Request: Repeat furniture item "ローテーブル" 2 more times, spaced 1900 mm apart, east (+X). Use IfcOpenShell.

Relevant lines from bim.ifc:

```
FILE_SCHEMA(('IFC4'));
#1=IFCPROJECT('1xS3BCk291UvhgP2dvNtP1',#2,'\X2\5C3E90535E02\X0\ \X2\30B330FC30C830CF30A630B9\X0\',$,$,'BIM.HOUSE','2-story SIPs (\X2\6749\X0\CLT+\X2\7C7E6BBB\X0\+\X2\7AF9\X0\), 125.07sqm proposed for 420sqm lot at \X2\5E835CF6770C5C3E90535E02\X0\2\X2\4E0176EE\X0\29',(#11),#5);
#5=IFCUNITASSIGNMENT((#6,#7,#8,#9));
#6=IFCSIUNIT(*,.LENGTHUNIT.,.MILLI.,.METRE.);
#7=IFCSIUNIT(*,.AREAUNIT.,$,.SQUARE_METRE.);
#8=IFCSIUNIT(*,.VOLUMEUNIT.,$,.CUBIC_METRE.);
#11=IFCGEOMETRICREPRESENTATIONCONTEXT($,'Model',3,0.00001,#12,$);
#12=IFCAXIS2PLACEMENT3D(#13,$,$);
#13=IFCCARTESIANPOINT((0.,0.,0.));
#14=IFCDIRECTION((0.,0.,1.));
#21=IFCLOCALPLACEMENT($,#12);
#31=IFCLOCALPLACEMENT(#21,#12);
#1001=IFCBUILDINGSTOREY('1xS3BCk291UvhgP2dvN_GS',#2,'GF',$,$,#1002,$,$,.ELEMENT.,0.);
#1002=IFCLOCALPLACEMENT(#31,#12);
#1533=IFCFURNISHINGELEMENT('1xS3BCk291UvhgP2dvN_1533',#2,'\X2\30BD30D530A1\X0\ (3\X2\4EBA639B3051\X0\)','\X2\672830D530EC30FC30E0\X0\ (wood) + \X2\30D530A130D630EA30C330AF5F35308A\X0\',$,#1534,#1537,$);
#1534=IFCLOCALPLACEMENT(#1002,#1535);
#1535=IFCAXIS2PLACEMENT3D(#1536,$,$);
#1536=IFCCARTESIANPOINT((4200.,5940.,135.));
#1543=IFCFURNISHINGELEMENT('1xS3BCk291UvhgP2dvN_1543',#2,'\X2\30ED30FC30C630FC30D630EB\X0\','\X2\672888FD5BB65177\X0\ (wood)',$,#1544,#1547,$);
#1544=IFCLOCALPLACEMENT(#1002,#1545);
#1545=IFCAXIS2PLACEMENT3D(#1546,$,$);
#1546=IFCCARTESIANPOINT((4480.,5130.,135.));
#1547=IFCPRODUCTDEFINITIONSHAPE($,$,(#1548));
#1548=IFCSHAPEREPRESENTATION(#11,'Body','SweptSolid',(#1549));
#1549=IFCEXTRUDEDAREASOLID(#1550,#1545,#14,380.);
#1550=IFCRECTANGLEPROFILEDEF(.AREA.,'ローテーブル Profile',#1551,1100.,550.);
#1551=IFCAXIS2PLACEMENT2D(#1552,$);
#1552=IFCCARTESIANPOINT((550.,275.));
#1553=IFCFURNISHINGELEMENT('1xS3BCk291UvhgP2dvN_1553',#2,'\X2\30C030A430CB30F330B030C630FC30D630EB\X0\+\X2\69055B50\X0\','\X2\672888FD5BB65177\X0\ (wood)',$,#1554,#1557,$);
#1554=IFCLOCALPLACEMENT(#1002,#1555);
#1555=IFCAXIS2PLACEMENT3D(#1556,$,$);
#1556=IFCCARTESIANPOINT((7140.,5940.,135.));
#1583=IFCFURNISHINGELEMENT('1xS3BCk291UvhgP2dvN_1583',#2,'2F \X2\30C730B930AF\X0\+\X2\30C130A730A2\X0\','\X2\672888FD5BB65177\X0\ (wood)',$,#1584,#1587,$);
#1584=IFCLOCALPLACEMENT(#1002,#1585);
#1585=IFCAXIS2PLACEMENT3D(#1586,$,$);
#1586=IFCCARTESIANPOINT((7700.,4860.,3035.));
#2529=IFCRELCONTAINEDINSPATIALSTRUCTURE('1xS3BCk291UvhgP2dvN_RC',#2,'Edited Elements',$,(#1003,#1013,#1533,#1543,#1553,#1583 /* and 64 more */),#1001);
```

```python
import numpy as np
import ifcopenshell
import ifcopenshell.api.geometry
import ifcopenshell.api.root
import ifcopenshell.util.element
import ifcopenshell.util.placement
import ifcopenshell.util.unit

model = ifcopenshell.open("bim.ifc")
unit_scale = ifcopenshell.util.unit.calculate_unit_scale(model)


def reuse_history(source, copy):
    """copy_class also copies each property set's owner history, people and application; keep the originals."""
    for rel in copy.IsDefinedBy:
        if rel.is_a("IfcRelDefinesByProperties") and (history := rel.RelatingPropertyDefinition.OwnerHistory):
            rel.RelatingPropertyDefinition.OwnerHistory = source.OwnerHistory
            ifcopenshell.util.element.remove_deep2(model, history)


source = model.by_guid("1xS3BCk291UvhgP2dvN_1543")
base = ifcopenshell.util.placement.get_local_placement(source.ObjectPlacement)
step = np.array([1.0, 0.0, 0.0]) * 1.9 / unit_scale

for i in range(1, 3):
    copy = ifcopenshell.api.root.copy_class(model, product=source)
    copy.Representation = ifcopenshell.util.element.copy_deep(
        model, source.Representation, exclude=["IfcGeometricRepresentationContext", "IfcRepresentationMap"]
    )
    reuse_history(source, copy)
    matrix = base.copy()
    matrix[:3, 3] += i * step
    print("added at", matrix[:3, 3].round(3) + 0.0)
    ifcopenshell.api.geometry.edit_object_placement(model, product=copy, matrix=matrix, is_si=False)

model.write("bim_rev.ifc")
```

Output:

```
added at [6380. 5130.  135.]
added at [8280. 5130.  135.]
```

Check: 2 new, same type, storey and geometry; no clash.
